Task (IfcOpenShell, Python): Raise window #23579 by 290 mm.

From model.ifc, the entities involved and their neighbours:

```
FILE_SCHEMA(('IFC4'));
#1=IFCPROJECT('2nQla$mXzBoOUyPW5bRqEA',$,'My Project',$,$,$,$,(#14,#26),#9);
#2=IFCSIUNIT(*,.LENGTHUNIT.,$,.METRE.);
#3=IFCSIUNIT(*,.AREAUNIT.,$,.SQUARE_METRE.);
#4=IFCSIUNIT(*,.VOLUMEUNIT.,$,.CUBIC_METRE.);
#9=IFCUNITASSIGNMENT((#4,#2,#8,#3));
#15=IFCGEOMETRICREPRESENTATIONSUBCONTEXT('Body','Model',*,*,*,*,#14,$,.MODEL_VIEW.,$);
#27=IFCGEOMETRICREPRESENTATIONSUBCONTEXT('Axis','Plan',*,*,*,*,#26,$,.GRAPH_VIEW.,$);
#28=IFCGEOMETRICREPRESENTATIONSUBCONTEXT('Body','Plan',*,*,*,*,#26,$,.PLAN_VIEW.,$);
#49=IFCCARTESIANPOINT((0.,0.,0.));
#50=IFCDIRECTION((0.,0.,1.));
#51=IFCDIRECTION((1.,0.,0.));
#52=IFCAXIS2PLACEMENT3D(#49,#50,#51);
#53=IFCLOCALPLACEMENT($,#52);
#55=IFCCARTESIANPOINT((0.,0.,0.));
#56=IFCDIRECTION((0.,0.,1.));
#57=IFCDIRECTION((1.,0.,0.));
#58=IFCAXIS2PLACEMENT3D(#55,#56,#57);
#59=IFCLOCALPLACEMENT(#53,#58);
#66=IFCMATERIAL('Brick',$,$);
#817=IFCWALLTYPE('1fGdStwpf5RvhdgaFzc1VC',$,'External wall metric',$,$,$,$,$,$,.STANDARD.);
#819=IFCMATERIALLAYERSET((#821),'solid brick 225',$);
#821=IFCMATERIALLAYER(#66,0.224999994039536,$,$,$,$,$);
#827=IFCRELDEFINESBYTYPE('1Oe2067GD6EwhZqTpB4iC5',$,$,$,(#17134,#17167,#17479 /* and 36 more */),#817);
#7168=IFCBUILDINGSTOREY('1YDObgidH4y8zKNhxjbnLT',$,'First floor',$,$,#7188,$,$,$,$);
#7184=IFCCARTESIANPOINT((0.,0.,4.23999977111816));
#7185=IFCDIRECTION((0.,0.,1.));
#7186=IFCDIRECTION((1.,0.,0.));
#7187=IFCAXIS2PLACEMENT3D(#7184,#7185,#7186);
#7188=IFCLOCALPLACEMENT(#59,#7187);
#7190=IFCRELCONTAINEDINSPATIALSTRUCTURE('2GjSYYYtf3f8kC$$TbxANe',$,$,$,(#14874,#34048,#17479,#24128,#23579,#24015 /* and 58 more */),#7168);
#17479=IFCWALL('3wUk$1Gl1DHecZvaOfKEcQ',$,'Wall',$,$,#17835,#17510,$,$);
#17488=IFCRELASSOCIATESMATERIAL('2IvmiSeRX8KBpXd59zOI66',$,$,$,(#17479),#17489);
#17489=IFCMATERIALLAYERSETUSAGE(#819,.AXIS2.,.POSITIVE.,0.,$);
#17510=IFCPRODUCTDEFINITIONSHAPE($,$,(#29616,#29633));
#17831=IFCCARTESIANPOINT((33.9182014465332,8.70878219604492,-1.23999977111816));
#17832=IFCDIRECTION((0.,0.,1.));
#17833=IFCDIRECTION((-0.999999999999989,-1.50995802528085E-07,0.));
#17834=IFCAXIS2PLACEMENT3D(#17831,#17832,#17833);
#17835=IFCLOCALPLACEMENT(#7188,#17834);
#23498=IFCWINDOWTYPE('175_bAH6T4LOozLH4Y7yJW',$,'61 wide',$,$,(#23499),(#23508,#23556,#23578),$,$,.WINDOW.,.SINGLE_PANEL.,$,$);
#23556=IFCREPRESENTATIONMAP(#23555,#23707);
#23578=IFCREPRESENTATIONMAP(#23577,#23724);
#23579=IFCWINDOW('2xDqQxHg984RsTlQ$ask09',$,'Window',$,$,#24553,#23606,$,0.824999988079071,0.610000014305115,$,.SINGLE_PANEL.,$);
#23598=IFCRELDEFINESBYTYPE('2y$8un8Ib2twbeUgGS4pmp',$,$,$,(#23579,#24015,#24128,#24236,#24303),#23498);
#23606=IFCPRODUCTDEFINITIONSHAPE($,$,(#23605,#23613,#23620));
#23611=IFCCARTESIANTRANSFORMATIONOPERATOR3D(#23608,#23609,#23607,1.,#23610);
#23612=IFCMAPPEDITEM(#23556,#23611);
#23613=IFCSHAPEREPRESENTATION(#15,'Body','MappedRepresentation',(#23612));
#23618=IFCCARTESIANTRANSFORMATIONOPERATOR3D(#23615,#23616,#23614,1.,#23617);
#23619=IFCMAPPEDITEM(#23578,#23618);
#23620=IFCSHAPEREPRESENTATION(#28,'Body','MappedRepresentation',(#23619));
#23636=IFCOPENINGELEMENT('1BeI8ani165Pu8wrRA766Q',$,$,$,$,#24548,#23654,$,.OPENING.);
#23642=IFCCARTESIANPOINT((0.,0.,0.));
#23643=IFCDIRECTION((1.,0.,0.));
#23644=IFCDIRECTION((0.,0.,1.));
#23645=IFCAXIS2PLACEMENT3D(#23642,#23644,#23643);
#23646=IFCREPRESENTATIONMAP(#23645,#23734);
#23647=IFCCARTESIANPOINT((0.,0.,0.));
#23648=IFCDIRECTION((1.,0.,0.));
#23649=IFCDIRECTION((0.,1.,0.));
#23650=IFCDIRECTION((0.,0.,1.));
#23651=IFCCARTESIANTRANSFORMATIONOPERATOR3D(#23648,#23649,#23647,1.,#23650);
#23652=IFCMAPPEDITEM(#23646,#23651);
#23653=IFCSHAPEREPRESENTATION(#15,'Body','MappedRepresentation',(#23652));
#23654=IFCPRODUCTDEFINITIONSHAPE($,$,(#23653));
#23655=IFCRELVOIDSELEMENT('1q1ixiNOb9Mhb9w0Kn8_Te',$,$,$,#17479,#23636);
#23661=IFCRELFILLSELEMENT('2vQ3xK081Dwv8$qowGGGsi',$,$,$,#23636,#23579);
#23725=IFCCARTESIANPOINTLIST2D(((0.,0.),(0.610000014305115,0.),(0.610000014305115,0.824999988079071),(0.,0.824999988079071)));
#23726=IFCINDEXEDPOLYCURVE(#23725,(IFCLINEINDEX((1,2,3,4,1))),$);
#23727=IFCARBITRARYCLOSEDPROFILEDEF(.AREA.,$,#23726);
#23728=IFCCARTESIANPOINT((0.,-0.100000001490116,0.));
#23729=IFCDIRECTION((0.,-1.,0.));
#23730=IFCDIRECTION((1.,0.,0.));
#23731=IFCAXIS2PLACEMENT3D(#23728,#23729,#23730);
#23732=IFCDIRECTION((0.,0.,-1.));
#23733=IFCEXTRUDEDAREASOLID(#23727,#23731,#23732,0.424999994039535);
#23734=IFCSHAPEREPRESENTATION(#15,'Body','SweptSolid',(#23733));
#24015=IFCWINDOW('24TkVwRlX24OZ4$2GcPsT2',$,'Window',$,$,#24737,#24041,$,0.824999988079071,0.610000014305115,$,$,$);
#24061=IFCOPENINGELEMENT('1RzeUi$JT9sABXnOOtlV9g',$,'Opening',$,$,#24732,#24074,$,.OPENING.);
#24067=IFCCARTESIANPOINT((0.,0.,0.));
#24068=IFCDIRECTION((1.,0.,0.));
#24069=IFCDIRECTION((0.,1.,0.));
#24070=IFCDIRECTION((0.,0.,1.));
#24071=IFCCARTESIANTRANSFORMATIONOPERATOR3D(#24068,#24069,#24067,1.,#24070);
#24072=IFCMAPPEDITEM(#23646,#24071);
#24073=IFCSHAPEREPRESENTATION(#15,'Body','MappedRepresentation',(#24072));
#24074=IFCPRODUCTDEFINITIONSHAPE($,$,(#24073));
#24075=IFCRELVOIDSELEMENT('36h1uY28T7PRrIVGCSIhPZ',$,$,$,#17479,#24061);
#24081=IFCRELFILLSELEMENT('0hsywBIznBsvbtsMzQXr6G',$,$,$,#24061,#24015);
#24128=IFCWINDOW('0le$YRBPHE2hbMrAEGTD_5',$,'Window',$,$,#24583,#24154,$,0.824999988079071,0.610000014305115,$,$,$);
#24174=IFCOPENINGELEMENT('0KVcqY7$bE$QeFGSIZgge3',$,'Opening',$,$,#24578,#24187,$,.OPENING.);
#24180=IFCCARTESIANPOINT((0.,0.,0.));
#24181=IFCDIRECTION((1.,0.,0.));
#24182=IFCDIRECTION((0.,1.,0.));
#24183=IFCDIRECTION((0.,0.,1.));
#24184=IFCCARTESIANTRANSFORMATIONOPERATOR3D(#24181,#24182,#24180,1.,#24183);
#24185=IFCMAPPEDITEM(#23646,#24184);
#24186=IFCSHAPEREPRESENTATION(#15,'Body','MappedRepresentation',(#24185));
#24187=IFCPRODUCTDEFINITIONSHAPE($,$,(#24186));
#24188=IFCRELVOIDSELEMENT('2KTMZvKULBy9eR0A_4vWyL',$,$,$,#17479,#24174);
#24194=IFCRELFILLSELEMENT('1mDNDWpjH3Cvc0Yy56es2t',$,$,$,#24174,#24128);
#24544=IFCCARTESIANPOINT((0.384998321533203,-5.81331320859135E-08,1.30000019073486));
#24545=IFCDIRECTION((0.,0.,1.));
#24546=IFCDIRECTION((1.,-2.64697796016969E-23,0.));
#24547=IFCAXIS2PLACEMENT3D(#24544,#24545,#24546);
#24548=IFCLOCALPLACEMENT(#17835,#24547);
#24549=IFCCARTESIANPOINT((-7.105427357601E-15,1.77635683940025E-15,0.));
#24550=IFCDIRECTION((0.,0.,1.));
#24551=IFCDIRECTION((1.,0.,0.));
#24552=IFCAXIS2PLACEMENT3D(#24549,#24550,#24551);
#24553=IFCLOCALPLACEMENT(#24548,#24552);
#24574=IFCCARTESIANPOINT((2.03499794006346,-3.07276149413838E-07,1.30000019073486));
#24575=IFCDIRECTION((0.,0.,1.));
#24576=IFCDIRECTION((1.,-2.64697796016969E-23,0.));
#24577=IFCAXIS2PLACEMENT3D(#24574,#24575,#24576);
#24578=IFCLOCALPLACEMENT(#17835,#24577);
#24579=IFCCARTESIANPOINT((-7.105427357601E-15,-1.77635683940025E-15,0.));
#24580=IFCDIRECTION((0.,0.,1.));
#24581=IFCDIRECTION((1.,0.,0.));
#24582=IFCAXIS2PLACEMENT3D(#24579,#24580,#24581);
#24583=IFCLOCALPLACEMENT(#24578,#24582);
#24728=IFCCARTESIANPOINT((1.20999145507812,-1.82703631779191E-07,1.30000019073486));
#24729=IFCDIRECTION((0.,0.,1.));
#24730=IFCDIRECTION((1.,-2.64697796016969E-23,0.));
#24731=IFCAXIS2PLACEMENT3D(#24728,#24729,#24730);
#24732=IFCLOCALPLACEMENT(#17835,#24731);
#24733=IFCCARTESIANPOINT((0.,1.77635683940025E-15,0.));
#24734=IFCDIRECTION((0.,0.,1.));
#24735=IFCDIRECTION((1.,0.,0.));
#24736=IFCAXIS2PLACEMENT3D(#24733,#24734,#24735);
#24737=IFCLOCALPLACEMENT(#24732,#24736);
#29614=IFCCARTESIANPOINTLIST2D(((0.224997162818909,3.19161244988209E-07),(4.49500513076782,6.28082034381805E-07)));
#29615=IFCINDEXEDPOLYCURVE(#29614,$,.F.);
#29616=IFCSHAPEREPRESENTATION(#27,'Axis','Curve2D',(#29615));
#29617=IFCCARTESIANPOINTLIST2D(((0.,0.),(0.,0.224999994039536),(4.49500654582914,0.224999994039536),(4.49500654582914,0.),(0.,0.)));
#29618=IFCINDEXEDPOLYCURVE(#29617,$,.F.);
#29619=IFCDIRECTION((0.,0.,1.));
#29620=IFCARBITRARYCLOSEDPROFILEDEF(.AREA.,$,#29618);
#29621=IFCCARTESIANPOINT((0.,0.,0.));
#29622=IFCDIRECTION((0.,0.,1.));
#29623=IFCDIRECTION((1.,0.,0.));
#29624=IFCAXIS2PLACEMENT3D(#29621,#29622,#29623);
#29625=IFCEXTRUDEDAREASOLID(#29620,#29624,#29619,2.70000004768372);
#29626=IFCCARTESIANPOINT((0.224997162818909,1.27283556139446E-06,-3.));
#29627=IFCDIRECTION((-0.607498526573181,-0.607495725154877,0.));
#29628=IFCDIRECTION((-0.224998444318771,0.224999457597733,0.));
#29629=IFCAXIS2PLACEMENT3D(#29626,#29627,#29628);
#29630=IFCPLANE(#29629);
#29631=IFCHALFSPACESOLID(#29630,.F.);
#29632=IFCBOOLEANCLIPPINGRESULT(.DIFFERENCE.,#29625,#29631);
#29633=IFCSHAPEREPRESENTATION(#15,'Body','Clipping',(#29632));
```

```python
import numpy as np
import ifcopenshell
import ifcopenshell.api.geometry
import ifcopenshell.util.placement
import ifcopenshell.util.unit

model = ifcopenshell.open("model.ifc")
unit_scale = ifcopenshell.util.unit.calculate_unit_scale(model)

window = model.by_id(23579)
opening = window.FillsVoids[0].RelatingOpeningElement
dz = 0.29 / unit_scale

shift = np.array([0.0, 0.0, dz])
# The window is placed relative to its opening, so it follows when the opening moves.
matrix = ifcopenshell.util.placement.get_local_placement(opening.ObjectPlacement)
matrix[:3, 3] += shift
ifcopenshell.api.geometry.edit_object_placement(
    model, product=opening, matrix=matrix, is_si=False, should_transform_children=True
)

print(f"moved by {dz * unit_scale:+.3f} m")

model.write("model_rev.ifc")
```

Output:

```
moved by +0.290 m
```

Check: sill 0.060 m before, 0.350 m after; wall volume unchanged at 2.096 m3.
